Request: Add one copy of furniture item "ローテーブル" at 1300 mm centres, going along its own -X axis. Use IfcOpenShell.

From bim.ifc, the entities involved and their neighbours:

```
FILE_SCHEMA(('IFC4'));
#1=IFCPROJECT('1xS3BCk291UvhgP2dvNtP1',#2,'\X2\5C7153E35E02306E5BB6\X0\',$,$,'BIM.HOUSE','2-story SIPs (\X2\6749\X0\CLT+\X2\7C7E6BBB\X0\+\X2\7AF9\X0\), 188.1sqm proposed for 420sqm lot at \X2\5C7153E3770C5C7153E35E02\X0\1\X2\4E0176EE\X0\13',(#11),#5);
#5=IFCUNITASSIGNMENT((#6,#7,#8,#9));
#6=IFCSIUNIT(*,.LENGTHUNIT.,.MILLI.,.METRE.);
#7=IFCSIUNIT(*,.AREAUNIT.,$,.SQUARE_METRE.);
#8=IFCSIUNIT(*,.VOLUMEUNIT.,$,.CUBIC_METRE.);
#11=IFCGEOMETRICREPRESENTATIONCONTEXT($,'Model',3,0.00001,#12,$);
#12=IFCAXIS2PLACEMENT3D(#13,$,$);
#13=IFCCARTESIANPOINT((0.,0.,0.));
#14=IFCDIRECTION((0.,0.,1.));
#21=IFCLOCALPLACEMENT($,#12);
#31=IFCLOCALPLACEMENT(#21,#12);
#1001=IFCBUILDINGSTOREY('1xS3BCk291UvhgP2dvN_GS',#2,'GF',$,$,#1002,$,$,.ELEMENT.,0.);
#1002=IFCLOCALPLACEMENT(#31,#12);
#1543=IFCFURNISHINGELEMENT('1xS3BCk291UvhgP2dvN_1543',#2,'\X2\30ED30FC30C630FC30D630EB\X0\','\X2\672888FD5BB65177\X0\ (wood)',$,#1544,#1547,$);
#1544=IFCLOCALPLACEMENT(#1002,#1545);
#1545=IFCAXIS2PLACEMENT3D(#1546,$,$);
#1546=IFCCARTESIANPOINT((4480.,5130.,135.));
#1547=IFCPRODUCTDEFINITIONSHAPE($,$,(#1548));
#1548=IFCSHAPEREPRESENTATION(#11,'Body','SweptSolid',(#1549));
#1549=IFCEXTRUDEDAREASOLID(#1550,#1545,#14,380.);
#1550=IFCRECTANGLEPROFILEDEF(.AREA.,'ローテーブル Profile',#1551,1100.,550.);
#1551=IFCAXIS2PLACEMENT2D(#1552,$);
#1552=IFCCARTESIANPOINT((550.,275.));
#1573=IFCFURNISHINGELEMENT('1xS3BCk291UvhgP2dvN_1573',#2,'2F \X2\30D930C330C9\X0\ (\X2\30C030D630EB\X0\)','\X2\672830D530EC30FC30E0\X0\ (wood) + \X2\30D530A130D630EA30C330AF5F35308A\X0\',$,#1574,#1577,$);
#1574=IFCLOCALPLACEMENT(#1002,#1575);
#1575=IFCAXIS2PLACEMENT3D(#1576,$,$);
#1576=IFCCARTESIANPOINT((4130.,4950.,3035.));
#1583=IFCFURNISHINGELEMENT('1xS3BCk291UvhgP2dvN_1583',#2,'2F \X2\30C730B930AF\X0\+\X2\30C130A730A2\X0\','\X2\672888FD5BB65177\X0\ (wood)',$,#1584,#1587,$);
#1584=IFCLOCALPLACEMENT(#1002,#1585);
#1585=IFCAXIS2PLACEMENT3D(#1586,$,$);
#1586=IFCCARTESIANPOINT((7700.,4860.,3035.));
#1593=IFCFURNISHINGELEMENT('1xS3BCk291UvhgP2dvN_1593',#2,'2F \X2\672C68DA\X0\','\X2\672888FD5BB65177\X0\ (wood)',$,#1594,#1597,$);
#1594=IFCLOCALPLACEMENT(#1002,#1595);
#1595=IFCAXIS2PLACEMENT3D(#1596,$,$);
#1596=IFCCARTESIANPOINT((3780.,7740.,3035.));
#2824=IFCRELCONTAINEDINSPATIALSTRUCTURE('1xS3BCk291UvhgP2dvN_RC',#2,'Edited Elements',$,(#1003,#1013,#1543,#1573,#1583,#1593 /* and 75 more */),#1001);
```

```python
import ifcopenshell
import ifcopenshell.api.geometry
import ifcopenshell.api.root
import ifcopenshell.util.element
import ifcopenshell.util.placement

model = ifcopenshell.open("bim.ifc")


def reuse_history(source, copy):
    """copy_class also copies each property set's owner history, people and application; keep the originals."""
    for rel in copy.IsDefinedBy:
        if rel.is_a("IfcRelDefinesByProperties") and (history := rel.RelatingPropertyDefinition.OwnerHistory):
            rel.RelatingPropertyDefinition.OwnerHistory = source.OwnerHistory
            ifcopenshell.util.element.remove_deep2(model, history)


source = model.by_guid("1xS3BCk291UvhgP2dvN_1543")
base = ifcopenshell.util.placement.get_local_placement(source.ObjectPlacement)
step = -base[:3, 0] * 1300.0

for i in range(1, 2):
    copy = ifcopenshell.api.root.copy_class(model, product=source)
    copy.Representation = ifcopenshell.util.element.copy_deep(
        model, source.Representation, exclude=["IfcGeometricRepresentationContext", "IfcRepresentationMap"]
    )
    reuse_history(source, copy)
    matrix = base.copy()
    matrix[:3, 3] += i * step
    print("added at", matrix[:3, 3].round(3) + 0.0)
    ifcopenshell.api.geometry.edit_object_placement(model, product=copy, matrix=matrix, is_si=False)

model.write("bim_v2.ifc")
```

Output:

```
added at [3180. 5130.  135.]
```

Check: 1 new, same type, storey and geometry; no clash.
